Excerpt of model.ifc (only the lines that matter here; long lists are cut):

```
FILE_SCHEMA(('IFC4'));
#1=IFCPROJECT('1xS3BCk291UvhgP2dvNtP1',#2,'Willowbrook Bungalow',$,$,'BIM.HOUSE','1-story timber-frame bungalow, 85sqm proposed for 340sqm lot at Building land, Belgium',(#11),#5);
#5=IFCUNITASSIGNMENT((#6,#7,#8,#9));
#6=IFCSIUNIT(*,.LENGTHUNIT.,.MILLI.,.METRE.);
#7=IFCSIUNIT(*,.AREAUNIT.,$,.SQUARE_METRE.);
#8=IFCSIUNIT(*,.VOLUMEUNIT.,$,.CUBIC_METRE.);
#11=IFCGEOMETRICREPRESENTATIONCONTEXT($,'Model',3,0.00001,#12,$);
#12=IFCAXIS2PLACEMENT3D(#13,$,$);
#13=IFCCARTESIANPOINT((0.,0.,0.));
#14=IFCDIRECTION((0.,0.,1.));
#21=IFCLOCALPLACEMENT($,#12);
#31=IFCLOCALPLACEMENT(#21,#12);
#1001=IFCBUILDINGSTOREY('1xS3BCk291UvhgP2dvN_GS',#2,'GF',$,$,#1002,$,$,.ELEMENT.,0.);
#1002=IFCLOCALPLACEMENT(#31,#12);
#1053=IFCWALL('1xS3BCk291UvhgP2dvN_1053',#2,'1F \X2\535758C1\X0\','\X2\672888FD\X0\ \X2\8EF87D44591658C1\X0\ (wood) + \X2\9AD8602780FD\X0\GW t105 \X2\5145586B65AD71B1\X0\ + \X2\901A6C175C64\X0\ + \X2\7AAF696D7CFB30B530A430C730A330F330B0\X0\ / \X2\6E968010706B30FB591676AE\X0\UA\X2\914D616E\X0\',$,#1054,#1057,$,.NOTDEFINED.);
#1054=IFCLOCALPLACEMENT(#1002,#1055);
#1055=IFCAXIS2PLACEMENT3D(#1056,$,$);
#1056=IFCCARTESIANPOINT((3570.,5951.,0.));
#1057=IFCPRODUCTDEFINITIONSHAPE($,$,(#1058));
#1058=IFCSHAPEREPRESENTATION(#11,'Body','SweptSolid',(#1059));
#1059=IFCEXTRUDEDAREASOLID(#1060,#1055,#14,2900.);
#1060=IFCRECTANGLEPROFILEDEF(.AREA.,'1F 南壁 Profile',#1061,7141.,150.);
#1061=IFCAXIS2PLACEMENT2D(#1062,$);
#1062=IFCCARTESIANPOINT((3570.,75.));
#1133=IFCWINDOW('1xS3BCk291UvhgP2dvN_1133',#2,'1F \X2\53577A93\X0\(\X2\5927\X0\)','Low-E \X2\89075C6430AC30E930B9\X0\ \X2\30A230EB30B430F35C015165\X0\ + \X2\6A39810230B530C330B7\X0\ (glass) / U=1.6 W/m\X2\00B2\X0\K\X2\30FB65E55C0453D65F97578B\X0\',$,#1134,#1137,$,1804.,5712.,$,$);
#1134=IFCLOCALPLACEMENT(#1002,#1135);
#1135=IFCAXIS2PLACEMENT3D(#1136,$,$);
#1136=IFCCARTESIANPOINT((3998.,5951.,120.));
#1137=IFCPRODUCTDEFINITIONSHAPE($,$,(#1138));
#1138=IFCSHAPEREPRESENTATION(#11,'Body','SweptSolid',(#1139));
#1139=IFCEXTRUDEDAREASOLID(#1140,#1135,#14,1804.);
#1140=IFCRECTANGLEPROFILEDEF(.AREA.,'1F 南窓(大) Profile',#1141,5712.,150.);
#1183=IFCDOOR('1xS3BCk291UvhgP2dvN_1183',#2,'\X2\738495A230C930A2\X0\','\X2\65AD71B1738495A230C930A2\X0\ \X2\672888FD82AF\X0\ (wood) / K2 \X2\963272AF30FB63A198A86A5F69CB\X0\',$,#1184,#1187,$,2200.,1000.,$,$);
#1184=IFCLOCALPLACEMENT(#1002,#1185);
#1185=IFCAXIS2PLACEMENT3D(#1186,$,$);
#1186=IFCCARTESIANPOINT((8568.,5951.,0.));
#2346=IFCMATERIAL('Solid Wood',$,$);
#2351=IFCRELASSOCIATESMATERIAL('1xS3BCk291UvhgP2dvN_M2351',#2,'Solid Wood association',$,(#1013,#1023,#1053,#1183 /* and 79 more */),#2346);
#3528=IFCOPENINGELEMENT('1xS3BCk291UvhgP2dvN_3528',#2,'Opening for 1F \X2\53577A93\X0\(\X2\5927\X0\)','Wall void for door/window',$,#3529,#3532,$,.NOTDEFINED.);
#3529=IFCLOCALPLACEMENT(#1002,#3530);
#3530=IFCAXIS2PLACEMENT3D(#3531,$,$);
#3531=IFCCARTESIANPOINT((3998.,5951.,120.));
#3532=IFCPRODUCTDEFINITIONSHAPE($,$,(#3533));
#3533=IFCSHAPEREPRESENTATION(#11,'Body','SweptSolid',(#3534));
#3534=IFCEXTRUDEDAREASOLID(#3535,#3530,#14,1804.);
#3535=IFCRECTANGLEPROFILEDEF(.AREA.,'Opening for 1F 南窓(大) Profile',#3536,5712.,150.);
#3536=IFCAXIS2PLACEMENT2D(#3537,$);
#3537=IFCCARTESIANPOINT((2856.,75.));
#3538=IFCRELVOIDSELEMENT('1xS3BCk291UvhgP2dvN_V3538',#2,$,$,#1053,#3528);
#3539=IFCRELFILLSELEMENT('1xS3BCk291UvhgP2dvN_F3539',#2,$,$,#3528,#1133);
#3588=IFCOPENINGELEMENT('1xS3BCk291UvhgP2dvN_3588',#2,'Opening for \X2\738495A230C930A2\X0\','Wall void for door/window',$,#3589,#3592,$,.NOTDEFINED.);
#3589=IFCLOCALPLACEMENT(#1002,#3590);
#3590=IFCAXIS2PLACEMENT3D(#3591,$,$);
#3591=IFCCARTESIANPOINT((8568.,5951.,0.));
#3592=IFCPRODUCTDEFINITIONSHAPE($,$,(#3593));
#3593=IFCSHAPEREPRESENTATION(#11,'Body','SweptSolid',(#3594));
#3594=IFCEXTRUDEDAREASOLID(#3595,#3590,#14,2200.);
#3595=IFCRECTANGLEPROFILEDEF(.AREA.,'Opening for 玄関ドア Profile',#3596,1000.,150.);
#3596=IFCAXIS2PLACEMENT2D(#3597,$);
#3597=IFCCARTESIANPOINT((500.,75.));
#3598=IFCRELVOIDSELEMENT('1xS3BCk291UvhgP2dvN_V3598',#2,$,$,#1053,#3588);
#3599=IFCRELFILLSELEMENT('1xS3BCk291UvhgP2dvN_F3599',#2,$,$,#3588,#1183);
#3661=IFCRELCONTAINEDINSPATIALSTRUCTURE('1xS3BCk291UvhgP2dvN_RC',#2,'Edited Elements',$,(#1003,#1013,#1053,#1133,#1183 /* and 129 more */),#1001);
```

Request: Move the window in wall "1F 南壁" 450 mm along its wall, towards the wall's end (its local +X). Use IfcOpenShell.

```python
import ifcopenshell
import ifcopenshell.api.geometry
import ifcopenshell.util.placement
import ifcopenshell.util.unit

model = ifcopenshell.open("model.ifc")
unit_scale = ifcopenshell.util.unit.calculate_unit_scale(model)

window = model.by_id(1133)
opening = window.FillsVoids[0].RelatingOpeningElement
wall = opening.VoidsElements[0].RelatingBuildingElement

wall_matrix = ifcopenshell.util.placement.get_local_placement(wall.ObjectPlacement)
shift = wall_matrix[:3, 0] * 0.45 / unit_scale
before = ifcopenshell.util.placement.get_local_placement(window.ObjectPlacement)[:3, 3].copy()

# The window is not placed relative to its opening, so move both.
for product in (opening, window):
    matrix = ifcopenshell.util.placement.get_local_placement(product.ObjectPlacement)
    matrix[:3, 3] += shift
    ifcopenshell.api.geometry.edit_object_placement(model, product=product, matrix=matrix, is_si=False)

after = ifcopenshell.util.placement.get_local_placement(window.ObjectPlacement)[:3, 3]
print("window moved by", (after - before).round(3) + 0.0)

model.write("model_updated.ifc")
```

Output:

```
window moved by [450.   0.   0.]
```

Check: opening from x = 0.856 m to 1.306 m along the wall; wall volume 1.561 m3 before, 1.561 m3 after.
